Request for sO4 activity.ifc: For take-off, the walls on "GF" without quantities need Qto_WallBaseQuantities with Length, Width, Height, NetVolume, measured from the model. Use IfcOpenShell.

First a look at what the model holds.

```python
import ifcopenshell
import ifcopenshell.util.element
import ifcopenshell.util.unit

model = ifcopenshell.open("sO4 activity.ifc")
print(model.schema)
for unit_type in ("LENGTHUNIT", "AREAUNIT", "VOLUMEUNIT"):
    print(unit_type, ifcopenshell.util.unit.calculate_unit_scale(model, unit_type))
storey = next(s for s in model.by_type("IfcBuildingStorey") if s.Name == "GF")
walls = [e for e in ifcopenshell.util.element.get_decomposition(storey) if e.is_a("IfcWall")]
for e in sorted(walls, key=lambda e: e.id()):
    print(e.id(), e.is_a(), e.Name, list(ifcopenshell.util.element.get_psets(e, qtos_only=True)), sep=" | ")
```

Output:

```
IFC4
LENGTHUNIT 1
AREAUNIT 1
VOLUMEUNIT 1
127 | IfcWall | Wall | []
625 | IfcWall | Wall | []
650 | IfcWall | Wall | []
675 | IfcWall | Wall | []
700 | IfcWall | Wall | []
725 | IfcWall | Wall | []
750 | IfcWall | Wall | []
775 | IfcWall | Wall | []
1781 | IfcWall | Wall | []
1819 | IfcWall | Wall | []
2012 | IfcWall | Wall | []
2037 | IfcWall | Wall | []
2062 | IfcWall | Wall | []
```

```python
import ifcopenshell
import ifcopenshell.api.pset
import ifcopenshell.geom
import ifcopenshell.util.element
import ifcopenshell.util.shape
import ifcopenshell.util.unit

model = ifcopenshell.open("sO4 activity.ifc")
unit_scale = ifcopenshell.util.unit.calculate_unit_scale(model)
volume_scale = ifcopenshell.util.unit.calculate_unit_scale(model, "VOLUMEUNIT")
settings = ifcopenshell.geom.settings()

storey = next(s for s in model.by_type("IfcBuildingStorey") if s.Name == "GF")
walls = [e for e in ifcopenshell.util.element.get_decomposition(storey) if e.is_a("IfcWall")]

for e in sorted(walls, key=lambda e: e.id()):
    if ifcopenshell.util.element.get_psets(e, qtos_only=True, should_inherit=False):
        continue
    # Geometry comes back in metres, in the element's own axes.
    shape = ifcopenshell.geom.create_shape(settings, e)
    values = {
        "Length": ifcopenshell.util.shape.get_x(shape.geometry) / unit_scale,
        "Width": ifcopenshell.util.shape.get_y(shape.geometry) / unit_scale,
        "Height": ifcopenshell.util.shape.get_z(shape.geometry) / unit_scale,
        "NetVolume": ifcopenshell.util.shape.get_volume(shape.geometry) / volume_scale,
    }
    qto = ifcopenshell.api.pset.add_qto(model, product=e, name="Qto_WallBaseQuantities")
    ifcopenshell.api.pset.edit_qto(model, qto=qto, properties=values)
    print(e.id(), {k: round(v, 3) for k, v in values.items()})

model.write("sO4 activity-out.ifc")
```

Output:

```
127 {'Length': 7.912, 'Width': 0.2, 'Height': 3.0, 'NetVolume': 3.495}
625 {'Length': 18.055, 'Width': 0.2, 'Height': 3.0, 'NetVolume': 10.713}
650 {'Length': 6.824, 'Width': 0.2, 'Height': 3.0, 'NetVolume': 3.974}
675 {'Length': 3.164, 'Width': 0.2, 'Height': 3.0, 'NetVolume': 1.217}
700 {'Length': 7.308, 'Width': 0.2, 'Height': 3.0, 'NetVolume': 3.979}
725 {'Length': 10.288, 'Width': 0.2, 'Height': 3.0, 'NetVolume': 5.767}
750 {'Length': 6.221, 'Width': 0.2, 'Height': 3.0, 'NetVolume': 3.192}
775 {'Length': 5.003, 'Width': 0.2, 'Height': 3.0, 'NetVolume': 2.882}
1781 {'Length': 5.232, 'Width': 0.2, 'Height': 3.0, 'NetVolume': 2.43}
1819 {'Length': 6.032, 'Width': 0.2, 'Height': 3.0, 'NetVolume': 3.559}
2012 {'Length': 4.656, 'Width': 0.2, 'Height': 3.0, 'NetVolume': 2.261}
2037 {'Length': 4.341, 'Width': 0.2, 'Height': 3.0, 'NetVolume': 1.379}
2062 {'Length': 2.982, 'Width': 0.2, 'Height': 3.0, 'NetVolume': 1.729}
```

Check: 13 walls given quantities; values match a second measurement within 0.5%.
